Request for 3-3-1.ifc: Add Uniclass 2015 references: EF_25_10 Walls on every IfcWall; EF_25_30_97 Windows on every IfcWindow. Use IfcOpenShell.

First a look at what the model holds.

```python
import ifcopenshell

model = ifcopenshell.open("3-3-1.ifc")
print(model.schema)
print("classifications:", [c.Name for c in model.by_type("IfcClassification")])
for ifc_class in ("IfcDoor", "IfcRoof", "IfcStair", "IfcWall", "IfcWindow"):
    print(ifc_class, len(model.by_type(ifc_class)))
```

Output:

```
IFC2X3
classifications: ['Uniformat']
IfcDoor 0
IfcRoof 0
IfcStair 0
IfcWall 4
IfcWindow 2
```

```python
import ifcopenshell
import ifcopenshell.api.classification

model = ifcopenshell.open("3-3-1.ifc")

# IFC2X3 requires Source and Edition and has no link from the project to the system.
system = model.create_entity("IfcClassification", Source="NBS", Edition="2015", Name="Uniclass 2015")

codes = {
    "IfcWall": ("EF_25_10", "Walls"),
    "IfcWindow": ("EF_25_30_97", "Windows"),
}
for ifc_class, (code, name) in codes.items():
    products = model.by_type(ifc_class)
    ifcopenshell.api.classification.add_reference(
        model, products=products, classification=system, identification=code, name=name
    )
    print(code, len(products))

model.write("3-3-1_updated.ifc")
```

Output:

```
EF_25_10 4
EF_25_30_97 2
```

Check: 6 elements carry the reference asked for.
